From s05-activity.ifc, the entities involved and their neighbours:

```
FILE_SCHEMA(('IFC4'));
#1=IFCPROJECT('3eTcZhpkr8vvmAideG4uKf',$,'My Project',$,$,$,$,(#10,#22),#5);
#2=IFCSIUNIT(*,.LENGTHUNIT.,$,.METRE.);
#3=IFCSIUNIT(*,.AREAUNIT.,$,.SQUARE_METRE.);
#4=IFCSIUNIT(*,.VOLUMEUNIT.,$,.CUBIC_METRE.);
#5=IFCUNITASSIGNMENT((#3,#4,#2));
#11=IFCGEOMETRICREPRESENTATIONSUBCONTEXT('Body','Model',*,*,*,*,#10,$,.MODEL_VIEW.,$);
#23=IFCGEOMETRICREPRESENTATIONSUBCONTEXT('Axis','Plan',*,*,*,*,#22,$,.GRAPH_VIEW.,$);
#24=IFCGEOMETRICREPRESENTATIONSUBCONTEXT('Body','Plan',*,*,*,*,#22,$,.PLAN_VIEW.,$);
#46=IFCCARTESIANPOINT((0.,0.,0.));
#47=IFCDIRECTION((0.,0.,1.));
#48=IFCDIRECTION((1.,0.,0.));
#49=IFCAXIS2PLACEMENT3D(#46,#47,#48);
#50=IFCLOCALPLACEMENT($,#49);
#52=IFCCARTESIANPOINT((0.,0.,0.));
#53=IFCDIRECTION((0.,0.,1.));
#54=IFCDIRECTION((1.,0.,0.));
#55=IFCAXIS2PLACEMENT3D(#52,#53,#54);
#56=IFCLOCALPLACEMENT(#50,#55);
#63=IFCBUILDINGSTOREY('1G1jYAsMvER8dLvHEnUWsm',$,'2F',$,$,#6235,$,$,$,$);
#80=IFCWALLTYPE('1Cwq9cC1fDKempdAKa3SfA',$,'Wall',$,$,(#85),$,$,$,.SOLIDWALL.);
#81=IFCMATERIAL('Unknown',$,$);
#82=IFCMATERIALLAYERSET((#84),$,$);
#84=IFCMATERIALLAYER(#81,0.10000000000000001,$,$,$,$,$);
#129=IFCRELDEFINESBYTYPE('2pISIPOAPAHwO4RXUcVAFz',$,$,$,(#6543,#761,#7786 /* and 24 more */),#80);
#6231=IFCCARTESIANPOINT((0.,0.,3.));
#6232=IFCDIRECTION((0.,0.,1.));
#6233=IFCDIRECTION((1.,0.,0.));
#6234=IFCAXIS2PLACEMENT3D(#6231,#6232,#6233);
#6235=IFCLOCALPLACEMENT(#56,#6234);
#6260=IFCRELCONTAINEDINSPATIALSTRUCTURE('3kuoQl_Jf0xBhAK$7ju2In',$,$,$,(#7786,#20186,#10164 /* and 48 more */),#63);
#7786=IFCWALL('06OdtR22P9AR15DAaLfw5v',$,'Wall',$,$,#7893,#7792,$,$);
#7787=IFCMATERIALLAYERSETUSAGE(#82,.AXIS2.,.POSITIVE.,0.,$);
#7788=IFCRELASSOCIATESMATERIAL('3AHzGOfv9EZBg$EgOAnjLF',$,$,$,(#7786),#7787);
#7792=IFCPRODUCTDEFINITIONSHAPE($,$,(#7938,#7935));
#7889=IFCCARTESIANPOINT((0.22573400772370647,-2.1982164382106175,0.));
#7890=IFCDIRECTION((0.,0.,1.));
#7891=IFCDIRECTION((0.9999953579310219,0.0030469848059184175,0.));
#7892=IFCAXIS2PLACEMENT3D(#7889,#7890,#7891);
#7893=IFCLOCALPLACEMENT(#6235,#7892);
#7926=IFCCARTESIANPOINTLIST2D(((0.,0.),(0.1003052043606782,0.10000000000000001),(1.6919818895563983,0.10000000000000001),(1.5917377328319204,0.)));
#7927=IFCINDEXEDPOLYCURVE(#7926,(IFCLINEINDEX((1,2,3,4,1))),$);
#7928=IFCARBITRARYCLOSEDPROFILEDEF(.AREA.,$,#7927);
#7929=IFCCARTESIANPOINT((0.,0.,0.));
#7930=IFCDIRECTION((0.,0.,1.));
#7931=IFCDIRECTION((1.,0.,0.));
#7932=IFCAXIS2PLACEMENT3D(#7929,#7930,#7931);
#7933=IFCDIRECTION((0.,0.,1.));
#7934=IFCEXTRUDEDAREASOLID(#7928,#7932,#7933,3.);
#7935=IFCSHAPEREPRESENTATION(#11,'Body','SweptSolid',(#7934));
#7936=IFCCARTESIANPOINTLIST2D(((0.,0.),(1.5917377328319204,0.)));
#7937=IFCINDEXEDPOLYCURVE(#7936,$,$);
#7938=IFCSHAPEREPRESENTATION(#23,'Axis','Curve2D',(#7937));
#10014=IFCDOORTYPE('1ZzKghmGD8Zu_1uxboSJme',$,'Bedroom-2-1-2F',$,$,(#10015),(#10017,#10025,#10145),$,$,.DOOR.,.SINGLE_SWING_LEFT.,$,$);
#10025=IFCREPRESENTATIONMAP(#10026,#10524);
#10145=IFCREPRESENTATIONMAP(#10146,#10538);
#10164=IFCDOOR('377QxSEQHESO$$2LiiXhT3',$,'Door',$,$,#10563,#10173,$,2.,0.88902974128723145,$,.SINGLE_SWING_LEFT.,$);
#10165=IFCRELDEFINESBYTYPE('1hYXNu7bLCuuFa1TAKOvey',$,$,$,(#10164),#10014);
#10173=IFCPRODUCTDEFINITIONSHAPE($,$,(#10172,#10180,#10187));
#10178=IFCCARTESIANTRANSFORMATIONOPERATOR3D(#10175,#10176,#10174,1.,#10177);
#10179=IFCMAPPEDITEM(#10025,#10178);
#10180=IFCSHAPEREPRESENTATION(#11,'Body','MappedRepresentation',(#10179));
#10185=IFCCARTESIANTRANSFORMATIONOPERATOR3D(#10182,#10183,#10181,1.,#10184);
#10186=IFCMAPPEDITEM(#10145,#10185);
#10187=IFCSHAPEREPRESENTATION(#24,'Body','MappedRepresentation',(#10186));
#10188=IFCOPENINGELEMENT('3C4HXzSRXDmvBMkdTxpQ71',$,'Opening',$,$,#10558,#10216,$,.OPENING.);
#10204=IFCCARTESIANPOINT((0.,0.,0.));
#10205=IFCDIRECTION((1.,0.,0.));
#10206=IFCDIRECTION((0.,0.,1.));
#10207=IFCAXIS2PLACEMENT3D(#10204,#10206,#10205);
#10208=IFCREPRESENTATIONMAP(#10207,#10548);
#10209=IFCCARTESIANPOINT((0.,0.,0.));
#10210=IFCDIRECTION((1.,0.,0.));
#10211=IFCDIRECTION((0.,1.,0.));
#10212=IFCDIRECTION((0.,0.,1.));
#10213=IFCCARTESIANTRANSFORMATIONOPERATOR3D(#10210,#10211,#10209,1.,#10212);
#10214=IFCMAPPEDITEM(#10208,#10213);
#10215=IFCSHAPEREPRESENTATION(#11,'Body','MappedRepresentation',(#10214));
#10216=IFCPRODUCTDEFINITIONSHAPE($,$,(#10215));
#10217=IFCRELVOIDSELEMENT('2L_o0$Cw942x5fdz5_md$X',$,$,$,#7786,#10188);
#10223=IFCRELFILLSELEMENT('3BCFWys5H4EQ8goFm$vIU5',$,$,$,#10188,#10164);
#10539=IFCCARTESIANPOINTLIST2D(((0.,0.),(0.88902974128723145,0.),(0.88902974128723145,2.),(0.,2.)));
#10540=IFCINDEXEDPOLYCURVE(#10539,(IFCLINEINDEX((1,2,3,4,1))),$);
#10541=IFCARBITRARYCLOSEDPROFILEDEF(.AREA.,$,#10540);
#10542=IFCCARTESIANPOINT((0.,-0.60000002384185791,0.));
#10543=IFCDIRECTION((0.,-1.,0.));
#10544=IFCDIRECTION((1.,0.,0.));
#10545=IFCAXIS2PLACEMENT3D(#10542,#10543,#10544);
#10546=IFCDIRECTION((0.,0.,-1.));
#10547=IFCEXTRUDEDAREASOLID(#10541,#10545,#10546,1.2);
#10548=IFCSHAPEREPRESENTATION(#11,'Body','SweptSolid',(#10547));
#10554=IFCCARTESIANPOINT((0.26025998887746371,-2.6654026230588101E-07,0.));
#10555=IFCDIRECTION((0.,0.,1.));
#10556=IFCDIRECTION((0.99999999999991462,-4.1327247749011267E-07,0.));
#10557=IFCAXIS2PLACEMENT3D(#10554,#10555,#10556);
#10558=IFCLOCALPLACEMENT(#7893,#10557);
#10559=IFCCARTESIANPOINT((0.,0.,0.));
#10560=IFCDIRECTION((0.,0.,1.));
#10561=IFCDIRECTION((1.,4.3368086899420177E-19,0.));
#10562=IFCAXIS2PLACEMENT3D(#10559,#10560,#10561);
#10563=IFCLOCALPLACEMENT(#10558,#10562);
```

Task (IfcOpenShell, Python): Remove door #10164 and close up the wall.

```python
import ifcopenshell
import ifcopenshell.api.feature
import ifcopenshell.api.root
import ifcopenshell.geom
import ifcopenshell.util.shape

model = ifcopenshell.open("s05-activity.ifc")
settings = ifcopenshell.geom.settings()


def volume(element):
    """Net volume in cubic metres, openings subtracted."""
    shape = ifcopenshell.geom.create_shape(settings, element)
    return ifcopenshell.util.shape.get_volume(shape.geometry)


door = model.by_guid("377QxSEQHESO$$2LiiXhT3")
opening = door.FillsVoids[0].RelatingOpeningElement
wall = opening.VoidsElements[0].RelatingBuildingElement
before = volume(wall)

ifcopenshell.api.root.remove_product(model, product=door)
ifcopenshell.api.feature.remove_feature(model, feature=opening)

after = volume(wall)

print(f"wall volume {before:.3f} -> {after:.3f} m3")

model.write("s05-activity_rev.ifc")
```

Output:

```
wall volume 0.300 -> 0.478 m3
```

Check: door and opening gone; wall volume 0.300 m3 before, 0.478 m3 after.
